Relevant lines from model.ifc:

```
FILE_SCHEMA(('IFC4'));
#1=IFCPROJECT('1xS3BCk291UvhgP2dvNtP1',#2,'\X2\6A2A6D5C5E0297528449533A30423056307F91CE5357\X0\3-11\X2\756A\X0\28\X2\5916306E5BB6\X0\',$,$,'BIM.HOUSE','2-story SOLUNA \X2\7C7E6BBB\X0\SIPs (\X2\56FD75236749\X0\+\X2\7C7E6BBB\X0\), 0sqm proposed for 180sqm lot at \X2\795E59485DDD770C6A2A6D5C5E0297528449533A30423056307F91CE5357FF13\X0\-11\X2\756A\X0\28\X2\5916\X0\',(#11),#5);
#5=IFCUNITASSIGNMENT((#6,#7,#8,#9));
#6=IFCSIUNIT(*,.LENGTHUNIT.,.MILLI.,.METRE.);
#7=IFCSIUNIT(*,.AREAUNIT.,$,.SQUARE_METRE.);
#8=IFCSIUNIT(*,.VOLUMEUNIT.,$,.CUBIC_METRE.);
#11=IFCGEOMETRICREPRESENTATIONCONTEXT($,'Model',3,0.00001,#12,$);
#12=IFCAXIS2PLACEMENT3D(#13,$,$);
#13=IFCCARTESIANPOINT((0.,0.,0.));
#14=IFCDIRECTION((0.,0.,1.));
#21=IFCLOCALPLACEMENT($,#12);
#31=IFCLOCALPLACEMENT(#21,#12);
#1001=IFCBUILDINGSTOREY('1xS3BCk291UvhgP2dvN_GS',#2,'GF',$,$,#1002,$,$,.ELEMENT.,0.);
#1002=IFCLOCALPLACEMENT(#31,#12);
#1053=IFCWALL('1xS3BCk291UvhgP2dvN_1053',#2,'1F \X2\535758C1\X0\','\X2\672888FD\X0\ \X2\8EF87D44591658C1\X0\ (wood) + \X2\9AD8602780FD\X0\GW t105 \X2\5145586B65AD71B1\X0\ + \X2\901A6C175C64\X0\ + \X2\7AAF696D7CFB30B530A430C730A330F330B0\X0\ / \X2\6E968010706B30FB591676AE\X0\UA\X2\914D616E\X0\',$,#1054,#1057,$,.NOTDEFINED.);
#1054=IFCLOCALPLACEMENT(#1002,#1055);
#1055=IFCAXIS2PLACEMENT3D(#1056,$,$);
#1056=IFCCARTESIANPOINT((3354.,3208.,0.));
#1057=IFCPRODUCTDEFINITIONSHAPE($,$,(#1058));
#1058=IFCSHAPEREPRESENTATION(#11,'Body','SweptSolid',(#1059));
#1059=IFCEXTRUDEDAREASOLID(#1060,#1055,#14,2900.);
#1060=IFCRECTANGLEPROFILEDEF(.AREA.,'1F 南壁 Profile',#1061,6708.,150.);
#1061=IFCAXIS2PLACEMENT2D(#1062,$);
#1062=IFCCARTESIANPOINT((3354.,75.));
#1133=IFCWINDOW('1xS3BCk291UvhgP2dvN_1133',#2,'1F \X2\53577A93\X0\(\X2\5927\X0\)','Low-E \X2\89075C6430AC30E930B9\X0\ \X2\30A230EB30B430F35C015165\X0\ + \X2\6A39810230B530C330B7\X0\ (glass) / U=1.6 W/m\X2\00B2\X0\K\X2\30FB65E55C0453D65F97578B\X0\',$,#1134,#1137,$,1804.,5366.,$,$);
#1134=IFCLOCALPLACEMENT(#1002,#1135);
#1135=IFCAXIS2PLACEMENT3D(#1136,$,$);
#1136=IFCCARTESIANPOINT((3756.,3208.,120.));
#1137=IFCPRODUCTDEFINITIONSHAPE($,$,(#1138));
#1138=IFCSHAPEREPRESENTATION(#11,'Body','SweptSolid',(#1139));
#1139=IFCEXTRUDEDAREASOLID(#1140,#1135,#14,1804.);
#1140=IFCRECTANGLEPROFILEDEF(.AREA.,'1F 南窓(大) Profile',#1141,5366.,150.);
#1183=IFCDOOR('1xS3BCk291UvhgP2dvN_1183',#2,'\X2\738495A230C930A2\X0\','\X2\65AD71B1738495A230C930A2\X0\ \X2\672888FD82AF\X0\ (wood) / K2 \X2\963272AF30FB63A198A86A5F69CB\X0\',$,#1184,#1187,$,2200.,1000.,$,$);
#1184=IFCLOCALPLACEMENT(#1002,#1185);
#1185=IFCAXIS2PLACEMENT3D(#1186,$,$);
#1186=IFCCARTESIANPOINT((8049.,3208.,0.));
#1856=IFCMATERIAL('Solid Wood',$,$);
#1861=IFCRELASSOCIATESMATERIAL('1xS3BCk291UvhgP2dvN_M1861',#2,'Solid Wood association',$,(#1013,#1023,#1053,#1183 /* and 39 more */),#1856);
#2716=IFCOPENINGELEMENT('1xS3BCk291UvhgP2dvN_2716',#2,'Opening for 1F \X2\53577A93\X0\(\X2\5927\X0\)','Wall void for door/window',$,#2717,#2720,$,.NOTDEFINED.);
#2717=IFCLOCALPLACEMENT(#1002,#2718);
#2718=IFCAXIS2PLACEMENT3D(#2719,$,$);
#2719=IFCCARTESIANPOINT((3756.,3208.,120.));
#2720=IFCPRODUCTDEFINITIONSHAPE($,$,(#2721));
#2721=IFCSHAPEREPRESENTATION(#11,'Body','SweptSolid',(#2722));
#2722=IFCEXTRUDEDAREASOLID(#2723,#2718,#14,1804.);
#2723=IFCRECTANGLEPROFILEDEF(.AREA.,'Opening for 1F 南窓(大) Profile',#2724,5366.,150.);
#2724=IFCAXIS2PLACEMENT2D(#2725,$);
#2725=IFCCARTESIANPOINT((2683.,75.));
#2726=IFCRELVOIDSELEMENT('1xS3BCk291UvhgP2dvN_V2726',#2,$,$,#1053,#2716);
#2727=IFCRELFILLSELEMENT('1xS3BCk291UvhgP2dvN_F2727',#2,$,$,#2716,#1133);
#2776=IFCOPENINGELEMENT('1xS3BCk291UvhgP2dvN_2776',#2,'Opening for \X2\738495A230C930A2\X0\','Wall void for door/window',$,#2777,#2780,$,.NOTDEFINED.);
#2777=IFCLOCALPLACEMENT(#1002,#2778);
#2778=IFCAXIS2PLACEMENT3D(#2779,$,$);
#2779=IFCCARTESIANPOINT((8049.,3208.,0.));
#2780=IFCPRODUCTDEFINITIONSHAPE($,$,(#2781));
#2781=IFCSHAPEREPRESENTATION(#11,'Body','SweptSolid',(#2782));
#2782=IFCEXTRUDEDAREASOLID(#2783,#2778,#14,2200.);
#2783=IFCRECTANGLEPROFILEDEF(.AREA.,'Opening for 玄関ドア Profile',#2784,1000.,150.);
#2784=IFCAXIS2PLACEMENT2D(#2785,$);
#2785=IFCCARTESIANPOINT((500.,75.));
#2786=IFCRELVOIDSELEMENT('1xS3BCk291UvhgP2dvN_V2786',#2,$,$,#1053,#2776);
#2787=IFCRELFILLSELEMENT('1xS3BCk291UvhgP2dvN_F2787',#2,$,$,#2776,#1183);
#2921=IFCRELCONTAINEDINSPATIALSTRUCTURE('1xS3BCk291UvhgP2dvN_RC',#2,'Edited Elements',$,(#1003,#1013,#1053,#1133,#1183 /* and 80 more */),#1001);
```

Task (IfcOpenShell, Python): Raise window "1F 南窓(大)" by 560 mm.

```python
import numpy as np
import ifcopenshell
import ifcopenshell.api.geometry
import ifcopenshell.util.placement
import ifcopenshell.util.unit

model = ifcopenshell.open("model.ifc")
unit_scale = ifcopenshell.util.unit.calculate_unit_scale(model)

window = model.by_id(1133)
opening = window.FillsVoids[0].RelatingOpeningElement
dz = 560.0

shift = np.array([0.0, 0.0, dz])
# The window is not placed relative to its opening, so move both.
for product in (opening, window):
    matrix = ifcopenshell.util.placement.get_local_placement(product.ObjectPlacement)
    matrix[:3, 3] += shift
    ifcopenshell.api.geometry.edit_object_placement(model, product=product, matrix=matrix, is_si=False)

print(f"moved by {dz * unit_scale:+.3f} m")

model.write("model-out.ifc")
```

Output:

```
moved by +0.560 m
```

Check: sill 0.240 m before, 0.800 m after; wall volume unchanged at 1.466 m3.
